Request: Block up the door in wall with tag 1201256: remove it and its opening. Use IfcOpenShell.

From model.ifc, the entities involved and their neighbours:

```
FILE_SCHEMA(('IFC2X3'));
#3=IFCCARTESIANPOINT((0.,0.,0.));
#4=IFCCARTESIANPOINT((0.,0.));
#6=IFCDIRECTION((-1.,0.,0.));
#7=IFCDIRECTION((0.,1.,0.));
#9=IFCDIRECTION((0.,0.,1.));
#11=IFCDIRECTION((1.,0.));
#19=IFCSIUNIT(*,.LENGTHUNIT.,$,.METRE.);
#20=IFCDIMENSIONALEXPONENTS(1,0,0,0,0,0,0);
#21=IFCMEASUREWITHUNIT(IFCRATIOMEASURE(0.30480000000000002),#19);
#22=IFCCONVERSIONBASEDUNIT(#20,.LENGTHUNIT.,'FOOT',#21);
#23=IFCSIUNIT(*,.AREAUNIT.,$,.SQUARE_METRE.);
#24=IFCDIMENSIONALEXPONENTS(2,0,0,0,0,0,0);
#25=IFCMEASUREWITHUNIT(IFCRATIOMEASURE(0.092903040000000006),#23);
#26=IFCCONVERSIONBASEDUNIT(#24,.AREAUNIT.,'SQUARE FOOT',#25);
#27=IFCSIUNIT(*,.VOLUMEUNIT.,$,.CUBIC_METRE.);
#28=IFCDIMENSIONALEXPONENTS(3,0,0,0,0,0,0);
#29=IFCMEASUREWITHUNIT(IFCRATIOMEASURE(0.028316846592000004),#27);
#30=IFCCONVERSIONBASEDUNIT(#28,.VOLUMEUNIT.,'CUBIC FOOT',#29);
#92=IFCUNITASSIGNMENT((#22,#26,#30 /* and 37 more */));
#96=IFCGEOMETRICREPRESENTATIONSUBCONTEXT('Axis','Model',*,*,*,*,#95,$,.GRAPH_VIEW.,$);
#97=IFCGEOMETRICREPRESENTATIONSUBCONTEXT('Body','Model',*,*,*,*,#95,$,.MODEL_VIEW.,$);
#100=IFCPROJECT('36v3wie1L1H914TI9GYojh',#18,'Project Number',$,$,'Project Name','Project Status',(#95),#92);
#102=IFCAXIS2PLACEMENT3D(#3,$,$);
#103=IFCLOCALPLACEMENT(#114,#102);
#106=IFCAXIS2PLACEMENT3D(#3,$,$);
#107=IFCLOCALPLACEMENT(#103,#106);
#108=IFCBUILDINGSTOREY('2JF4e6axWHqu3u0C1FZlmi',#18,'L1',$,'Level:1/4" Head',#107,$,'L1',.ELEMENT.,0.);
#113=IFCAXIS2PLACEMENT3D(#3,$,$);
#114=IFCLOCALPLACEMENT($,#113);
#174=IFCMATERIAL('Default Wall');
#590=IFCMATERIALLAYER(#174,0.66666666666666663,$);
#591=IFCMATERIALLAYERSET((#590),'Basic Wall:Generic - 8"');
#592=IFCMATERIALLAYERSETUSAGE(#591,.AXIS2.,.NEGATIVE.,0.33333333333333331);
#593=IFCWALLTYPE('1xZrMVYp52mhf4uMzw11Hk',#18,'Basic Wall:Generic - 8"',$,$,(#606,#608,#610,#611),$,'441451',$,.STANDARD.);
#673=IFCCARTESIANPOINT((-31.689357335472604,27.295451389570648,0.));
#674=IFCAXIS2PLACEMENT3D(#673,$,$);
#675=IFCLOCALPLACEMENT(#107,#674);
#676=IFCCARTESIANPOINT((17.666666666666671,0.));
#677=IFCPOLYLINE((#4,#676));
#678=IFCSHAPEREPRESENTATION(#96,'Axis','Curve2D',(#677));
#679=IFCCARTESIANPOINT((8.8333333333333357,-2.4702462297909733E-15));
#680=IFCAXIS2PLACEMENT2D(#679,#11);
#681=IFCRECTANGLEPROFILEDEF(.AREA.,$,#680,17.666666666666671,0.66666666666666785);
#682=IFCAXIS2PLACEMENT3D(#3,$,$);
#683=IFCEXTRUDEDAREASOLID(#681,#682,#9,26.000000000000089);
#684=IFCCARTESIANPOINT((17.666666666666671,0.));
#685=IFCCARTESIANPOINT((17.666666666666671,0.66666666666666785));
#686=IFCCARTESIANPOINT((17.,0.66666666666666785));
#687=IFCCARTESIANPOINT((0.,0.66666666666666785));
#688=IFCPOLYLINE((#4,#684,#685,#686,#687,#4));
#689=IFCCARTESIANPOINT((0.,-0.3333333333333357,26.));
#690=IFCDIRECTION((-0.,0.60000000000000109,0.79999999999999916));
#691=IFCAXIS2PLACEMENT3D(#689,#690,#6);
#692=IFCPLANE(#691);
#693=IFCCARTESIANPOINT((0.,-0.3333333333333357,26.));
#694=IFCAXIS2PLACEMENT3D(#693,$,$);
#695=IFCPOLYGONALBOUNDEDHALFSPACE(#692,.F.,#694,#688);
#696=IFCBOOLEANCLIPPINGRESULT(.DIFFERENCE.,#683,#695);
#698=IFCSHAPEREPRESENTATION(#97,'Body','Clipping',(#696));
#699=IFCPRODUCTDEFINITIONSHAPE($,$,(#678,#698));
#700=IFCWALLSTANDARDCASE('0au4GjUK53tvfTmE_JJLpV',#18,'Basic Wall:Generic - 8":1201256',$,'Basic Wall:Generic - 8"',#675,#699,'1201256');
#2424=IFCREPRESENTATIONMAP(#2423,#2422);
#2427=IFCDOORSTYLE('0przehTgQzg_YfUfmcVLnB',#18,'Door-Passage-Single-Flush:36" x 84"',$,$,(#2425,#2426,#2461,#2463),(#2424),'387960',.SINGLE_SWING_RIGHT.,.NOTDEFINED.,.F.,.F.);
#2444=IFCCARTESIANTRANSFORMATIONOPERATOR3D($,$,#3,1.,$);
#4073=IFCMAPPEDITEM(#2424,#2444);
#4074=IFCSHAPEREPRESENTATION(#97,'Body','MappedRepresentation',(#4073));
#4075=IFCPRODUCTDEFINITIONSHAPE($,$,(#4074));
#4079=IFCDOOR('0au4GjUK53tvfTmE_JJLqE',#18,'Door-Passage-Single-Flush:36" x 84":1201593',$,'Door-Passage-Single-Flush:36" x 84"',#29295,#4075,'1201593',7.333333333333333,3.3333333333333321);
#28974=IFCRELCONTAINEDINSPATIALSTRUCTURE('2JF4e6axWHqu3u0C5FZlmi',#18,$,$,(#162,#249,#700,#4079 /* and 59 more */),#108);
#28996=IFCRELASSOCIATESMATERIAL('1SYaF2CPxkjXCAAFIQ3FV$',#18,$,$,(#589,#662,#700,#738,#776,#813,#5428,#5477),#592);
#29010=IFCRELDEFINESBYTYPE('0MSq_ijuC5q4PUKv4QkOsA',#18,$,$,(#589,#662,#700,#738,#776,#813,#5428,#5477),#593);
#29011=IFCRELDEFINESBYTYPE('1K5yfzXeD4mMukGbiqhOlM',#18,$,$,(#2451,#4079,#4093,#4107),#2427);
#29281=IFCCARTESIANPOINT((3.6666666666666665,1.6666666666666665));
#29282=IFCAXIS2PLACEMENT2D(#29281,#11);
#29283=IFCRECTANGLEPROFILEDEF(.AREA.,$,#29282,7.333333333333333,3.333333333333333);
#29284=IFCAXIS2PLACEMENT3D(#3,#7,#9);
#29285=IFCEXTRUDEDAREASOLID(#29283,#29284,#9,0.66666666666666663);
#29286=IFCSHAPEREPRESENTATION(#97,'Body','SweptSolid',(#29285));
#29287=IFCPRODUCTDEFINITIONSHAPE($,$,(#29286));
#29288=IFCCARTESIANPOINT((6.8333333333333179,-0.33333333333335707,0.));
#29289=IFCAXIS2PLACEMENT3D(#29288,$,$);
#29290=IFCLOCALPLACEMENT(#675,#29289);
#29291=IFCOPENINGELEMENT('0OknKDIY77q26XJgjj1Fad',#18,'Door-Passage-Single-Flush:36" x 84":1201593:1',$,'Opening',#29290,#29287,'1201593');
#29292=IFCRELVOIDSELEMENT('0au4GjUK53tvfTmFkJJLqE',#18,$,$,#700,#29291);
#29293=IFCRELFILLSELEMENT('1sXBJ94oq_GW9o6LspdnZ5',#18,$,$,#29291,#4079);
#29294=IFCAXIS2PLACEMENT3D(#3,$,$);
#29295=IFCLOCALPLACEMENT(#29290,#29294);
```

```python
import ifcopenshell
import ifcopenshell.api.feature
import ifcopenshell.api.root
import ifcopenshell.geom
import ifcopenshell.util.shape

model = ifcopenshell.open("model.ifc")
settings = ifcopenshell.geom.settings()


def volume(element):
    """Net volume in cubic metres, openings subtracted."""
    shape = ifcopenshell.geom.create_shape(settings, element)
    return ifcopenshell.util.shape.get_volume(shape.geometry)


door = model.by_guid("0au4GjUK53tvfTmE_JJLqE")
opening = door.FillsVoids[0].RelatingOpeningElement
wall = opening.VoidsElements[0].RelatingBuildingElement
before = volume(wall)

ifcopenshell.api.root.remove_product(model, product=door)
ifcopenshell.api.feature.remove_feature(model, feature=opening)

after = volume(wall)

print(f"wall volume {before:.3f} -> {after:.3f} m3")

model.write("model_rev.ifc")
```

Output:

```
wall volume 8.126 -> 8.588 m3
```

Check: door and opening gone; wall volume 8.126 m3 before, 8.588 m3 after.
